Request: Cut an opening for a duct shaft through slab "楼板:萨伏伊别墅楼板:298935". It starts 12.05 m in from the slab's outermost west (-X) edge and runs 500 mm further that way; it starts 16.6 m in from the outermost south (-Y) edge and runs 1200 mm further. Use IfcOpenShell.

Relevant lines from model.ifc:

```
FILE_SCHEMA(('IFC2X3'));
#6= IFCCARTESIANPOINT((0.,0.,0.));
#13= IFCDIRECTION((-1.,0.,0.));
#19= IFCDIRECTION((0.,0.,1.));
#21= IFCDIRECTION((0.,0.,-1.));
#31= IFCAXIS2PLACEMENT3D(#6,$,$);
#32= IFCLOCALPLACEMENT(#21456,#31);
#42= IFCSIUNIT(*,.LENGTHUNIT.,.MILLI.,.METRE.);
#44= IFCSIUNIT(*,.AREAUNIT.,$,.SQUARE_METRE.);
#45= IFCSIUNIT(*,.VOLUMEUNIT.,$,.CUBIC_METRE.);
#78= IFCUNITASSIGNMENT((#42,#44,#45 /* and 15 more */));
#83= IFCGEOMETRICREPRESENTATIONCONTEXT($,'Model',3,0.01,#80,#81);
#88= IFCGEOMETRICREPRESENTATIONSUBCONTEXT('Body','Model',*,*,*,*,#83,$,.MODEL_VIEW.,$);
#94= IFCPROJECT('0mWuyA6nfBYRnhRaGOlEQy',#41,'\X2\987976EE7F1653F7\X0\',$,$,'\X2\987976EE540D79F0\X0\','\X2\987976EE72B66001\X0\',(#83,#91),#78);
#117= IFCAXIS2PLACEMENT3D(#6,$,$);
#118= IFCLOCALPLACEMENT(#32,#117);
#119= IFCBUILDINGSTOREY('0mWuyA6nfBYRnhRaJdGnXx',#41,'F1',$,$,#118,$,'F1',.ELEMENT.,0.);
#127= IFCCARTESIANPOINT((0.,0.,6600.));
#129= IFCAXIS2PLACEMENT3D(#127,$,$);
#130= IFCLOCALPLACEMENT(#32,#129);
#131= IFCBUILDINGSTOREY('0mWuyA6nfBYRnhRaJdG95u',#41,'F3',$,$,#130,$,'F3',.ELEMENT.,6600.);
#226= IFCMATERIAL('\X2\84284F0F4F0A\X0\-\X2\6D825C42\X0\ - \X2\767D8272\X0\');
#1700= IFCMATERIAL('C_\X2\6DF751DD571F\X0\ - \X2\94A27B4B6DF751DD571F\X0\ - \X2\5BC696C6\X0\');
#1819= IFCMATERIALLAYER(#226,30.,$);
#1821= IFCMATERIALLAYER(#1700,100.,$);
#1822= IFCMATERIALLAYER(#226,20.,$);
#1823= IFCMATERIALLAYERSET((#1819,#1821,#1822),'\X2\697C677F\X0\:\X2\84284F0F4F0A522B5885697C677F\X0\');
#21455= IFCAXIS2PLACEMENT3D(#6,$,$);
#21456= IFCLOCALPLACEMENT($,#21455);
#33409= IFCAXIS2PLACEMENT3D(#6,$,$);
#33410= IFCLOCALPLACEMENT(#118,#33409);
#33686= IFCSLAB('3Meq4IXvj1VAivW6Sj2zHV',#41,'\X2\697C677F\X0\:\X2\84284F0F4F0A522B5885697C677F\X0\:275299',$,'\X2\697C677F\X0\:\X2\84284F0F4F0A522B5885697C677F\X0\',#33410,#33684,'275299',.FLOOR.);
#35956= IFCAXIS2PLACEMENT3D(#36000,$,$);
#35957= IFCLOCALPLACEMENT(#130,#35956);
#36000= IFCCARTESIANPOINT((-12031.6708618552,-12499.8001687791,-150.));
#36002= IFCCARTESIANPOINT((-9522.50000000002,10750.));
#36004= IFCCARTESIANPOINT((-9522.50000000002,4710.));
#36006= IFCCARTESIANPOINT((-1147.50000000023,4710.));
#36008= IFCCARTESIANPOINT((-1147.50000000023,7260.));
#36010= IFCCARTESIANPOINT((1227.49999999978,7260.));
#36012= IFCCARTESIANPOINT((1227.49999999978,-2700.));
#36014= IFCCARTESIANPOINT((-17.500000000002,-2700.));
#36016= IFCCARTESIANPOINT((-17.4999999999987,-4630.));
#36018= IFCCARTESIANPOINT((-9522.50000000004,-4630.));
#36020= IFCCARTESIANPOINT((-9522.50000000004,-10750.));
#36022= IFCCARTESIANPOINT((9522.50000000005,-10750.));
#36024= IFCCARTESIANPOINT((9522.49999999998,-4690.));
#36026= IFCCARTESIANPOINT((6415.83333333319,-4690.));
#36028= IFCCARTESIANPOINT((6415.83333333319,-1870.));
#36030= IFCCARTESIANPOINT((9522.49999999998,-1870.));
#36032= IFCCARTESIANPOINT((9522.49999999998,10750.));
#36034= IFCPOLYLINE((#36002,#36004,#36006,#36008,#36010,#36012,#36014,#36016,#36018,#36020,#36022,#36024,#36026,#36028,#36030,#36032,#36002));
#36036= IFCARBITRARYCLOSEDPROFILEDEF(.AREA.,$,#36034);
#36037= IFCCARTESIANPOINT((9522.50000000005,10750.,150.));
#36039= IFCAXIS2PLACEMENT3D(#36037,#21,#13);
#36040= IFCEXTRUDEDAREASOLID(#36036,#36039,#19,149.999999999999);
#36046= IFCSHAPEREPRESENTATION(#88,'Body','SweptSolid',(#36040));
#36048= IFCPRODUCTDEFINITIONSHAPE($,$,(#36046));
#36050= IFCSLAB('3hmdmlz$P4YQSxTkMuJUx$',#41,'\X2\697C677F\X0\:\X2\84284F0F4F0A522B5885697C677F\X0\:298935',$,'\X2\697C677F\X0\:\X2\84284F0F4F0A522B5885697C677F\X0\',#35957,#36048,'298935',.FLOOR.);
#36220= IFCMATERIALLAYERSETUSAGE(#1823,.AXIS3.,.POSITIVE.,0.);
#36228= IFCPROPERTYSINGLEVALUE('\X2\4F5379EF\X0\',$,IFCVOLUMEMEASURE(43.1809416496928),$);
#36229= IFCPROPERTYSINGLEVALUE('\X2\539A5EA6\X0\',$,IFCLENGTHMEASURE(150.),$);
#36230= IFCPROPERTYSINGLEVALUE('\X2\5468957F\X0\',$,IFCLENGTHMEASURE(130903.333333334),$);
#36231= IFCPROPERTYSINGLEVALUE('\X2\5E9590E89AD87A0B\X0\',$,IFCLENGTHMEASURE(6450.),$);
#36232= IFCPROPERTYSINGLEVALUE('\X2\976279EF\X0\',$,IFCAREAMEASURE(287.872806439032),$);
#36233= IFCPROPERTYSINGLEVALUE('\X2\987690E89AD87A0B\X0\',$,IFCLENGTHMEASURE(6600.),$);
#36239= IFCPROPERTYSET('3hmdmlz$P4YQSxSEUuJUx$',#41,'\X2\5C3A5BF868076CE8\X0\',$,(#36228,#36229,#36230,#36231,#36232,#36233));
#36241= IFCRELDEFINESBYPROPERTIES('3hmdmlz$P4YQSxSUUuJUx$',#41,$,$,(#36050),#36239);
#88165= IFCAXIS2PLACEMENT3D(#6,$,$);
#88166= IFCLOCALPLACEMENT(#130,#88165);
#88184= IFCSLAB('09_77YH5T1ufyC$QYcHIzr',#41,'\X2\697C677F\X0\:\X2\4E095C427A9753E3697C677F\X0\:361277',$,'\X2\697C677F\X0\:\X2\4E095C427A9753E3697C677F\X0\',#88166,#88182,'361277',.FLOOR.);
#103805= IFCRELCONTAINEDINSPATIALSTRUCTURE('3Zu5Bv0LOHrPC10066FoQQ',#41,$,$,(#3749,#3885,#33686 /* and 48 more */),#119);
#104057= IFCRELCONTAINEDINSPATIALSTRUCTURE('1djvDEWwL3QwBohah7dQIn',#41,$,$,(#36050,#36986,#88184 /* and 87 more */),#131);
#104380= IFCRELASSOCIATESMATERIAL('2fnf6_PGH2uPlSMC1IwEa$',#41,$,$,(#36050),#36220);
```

```python
import numpy as np
import ifcopenshell
import ifcopenshell.api.feature
import ifcopenshell.api.geometry
import ifcopenshell.api.pset
import ifcopenshell.api.root
import ifcopenshell.geom
import ifcopenshell.util.element
import ifcopenshell.util.placement
import ifcopenshell.util.representation
import ifcopenshell.util.shape
import ifcopenshell.util.unit

model = ifcopenshell.open("model.ifc")
unit_scale = ifcopenshell.util.unit.calculate_unit_scale(model)
area_scale = ifcopenshell.util.unit.calculate_unit_scale(model, "AREAUNIT")
volume_scale = ifcopenshell.util.unit.calculate_unit_scale(model, "VOLUMEUNIT")
settings = ifcopenshell.geom.settings()


def volume(element):
    """Net volume in cubic metres, openings subtracted."""
    shape = ifcopenshell.geom.create_shape(settings, element)
    return ifcopenshell.util.shape.get_volume(shape.geometry)


slab = model.by_guid("3hmdmlz$P4YQSxTkMuJUx$")
before = volume(slab)

# Extent in the slab's own axes, in metres. The edges named are its -X and -Y sides.
slab_shape = ifcopenshell.geom.create_shape(settings, slab)
vertices = ifcopenshell.util.shape.get_vertices(slab_shape.geometry)
x_min, y_min, bottom = vertices.min(axis=0)
top = vertices[:, 2].max()

opening = ifcopenshell.api.root.create_entity(model, ifc_class="IfcOpeningElement", name="Duct shaft opening")
context = ifcopenshell.util.representation.get_context(model, "Model", "Body", "MODEL_VIEW")
width, depth = 0.5, 1.2
outline = [(0.0, 0.0), (width, 0.0), (width, depth), (0.0, depth), (0.0, 0.0)]
# Overshoot both faces by 50 mm so the cut is clean.
shape = ifcopenshell.api.geometry.add_slab_representation(
    model, context=context, depth=top - bottom + 0.1, polyline=outline
)
ifcopenshell.api.geometry.assign_representation(model, product=opening, representation=shape)

matrix = ifcopenshell.util.placement.get_local_placement(slab.ObjectPlacement)
matrix[:, 3] = matrix @ np.append(np.array([x_min + 12.05, y_min + 16.6, bottom - 0.05]) / unit_scale, 1.0)
ifcopenshell.api.geometry.edit_object_placement(model, product=opening, matrix=matrix, is_si=False)
ifcopenshell.api.feature.add_feature(model, feature=opening, element=slab)

after = volume(slab)

# Update the slab's stored quantities.
pset = model.by_id(ifcopenshell.util.element.get_pset(slab, "尺寸标注", should_inherit=False)["id"])
ifcopenshell.api.pset.edit_pset(model, pset=pset, properties={
    "体积": model.create_entity("IfcVolumeMeasure", after / volume_scale),
    "面积": model.create_entity("IfcAreaMeasure", after / (top - bottom) / area_scale),
})

print(f"slab volume {before:.3f} -> {after:.3f} m3")

model.write("model_rev.ifc")
```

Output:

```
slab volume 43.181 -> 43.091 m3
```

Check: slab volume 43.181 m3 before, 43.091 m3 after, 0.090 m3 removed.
